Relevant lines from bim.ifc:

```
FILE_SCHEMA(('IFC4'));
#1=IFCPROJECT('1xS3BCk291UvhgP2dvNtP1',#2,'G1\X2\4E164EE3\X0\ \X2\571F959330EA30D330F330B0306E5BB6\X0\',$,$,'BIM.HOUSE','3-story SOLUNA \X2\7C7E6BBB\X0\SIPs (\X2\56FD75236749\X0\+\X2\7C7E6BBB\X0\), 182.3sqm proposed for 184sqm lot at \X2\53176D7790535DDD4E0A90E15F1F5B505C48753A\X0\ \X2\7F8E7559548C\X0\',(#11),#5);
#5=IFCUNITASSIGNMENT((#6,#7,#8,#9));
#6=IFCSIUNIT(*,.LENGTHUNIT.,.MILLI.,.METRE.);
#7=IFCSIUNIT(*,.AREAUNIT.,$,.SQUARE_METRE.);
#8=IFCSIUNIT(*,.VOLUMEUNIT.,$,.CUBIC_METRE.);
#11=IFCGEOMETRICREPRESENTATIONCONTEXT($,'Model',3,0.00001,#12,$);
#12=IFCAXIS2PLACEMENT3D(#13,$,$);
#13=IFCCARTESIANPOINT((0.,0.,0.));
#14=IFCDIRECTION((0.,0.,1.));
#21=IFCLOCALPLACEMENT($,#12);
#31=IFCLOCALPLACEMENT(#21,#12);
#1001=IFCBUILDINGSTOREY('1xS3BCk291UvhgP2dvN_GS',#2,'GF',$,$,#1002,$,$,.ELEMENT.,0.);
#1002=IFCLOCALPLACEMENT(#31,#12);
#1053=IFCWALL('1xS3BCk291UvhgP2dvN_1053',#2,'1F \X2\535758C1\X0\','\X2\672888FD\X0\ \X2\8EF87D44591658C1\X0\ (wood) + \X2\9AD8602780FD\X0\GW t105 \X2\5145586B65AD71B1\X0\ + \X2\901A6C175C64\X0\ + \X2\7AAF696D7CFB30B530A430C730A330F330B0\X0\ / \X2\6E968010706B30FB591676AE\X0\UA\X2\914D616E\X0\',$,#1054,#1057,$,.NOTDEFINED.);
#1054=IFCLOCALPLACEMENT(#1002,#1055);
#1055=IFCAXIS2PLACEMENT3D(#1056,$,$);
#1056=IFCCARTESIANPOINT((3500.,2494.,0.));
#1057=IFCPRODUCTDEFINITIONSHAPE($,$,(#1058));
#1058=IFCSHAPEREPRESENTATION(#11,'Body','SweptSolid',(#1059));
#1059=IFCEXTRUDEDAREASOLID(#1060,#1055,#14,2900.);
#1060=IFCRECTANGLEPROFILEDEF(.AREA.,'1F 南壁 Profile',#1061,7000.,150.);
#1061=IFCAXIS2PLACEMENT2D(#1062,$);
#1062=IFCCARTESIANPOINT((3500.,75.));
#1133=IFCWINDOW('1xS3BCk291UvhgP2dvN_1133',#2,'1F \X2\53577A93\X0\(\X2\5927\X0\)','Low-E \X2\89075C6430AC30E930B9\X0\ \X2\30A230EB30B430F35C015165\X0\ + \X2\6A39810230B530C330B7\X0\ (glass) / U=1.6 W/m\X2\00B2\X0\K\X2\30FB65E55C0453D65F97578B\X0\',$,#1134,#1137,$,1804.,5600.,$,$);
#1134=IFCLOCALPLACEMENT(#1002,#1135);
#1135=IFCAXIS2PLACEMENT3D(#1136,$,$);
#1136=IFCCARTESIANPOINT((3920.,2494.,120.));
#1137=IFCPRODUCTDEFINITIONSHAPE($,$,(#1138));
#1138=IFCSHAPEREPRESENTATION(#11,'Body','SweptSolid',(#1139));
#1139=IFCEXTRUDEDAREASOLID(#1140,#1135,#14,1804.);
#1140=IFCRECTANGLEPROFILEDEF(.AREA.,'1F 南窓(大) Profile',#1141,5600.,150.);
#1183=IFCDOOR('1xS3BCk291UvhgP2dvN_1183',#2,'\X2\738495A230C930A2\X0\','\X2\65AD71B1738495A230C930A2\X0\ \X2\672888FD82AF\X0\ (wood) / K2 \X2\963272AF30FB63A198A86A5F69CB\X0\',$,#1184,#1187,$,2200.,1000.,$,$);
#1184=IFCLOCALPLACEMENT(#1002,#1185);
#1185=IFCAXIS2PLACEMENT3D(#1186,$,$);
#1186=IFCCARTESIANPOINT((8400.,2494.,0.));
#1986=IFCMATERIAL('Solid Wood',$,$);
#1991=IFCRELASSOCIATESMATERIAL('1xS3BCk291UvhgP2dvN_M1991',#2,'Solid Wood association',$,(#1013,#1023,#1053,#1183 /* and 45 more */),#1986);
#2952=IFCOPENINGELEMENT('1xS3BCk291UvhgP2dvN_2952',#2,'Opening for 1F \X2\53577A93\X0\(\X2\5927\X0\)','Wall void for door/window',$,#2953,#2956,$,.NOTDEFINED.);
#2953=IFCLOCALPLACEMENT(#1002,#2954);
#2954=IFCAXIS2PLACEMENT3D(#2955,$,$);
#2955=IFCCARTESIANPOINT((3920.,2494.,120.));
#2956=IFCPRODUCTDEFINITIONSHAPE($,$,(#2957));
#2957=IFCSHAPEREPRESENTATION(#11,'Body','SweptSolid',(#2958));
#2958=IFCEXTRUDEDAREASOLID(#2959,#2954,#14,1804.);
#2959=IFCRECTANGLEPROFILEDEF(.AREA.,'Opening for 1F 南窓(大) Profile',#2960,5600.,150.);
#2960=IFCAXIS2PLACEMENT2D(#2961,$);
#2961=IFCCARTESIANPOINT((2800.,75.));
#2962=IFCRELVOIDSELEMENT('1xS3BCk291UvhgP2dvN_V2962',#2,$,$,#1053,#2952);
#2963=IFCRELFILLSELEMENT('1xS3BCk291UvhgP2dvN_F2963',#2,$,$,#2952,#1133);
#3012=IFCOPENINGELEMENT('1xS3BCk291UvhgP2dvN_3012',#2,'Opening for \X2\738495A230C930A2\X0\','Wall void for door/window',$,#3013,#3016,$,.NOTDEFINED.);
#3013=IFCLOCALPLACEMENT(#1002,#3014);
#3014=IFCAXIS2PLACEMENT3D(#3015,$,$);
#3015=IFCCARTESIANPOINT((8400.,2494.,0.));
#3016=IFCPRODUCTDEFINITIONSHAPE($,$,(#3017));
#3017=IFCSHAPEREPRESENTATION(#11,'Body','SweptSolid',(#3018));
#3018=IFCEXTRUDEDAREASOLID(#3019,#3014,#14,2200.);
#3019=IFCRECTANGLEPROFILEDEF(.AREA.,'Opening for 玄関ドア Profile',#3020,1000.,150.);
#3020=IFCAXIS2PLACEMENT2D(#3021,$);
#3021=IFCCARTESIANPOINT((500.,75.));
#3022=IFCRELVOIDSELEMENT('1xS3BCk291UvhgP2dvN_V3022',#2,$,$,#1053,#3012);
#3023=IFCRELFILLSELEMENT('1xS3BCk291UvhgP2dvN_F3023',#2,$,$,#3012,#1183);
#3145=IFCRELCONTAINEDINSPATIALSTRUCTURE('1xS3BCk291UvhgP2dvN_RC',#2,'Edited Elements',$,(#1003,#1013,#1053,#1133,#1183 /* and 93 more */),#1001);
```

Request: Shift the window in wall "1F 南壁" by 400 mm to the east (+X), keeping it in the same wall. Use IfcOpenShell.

```python
import ifcopenshell
import ifcopenshell.api.geometry
import ifcopenshell.util.placement

model = ifcopenshell.open("bim.ifc")

window = model.by_guid("1xS3BCk291UvhgP2dvN_1133")
opening = window.FillsVoids[0].RelatingOpeningElement
wall = opening.VoidsElements[0].RelatingBuildingElement

wall_matrix = ifcopenshell.util.placement.get_local_placement(wall.ObjectPlacement)
shift = wall_matrix[:3, 0] * 400.0
before = ifcopenshell.util.placement.get_local_placement(window.ObjectPlacement)[:3, 3].copy()

# The window is not placed relative to its opening, so move both.
for product in (opening, window):
    matrix = ifcopenshell.util.placement.get_local_placement(product.ObjectPlacement)
    matrix[:3, 3] += shift
    ifcopenshell.api.geometry.edit_object_placement(model, product=product, matrix=matrix, is_si=False)

after = ifcopenshell.util.placement.get_local_placement(window.ObjectPlacement)[:3, 3]
print("window moved by", (after - before).round(3) + 0.0)

model.write("bim_updated.ifc")
```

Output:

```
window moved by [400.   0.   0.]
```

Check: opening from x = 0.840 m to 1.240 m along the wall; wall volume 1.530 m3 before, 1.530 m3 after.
